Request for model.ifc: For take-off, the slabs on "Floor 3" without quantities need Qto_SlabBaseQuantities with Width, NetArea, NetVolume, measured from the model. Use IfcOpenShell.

First a look at what the model holds.

```python
import ifcopenshell
import ifcopenshell.util.element
import ifcopenshell.util.unit

model = ifcopenshell.open("model.ifc")
print(model.schema)
for unit_type in ("LENGTHUNIT", "AREAUNIT", "VOLUMEUNIT"):
    print(unit_type, ifcopenshell.util.unit.calculate_unit_scale(model, unit_type))
storey = next(s for s in model.by_type("IfcBuildingStorey") if s.Name == "Floor 3")
slabs = [e for e in ifcopenshell.util.element.get_decomposition(storey) if e.is_a("IfcSlab")]
for e in sorted(slabs, key=lambda e: e.id()):
    print(e.id(), e.is_a(), e.Name, list(ifcopenshell.util.element.get_psets(e, qtos_only=True)), sep=" | ")
```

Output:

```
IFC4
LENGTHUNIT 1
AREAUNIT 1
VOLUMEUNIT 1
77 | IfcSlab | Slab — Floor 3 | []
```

```python
import ifcopenshell
import ifcopenshell.api.pset
import ifcopenshell.geom
import ifcopenshell.util.element
import ifcopenshell.util.shape
import ifcopenshell.util.unit

model = ifcopenshell.open("model.ifc")
unit_scale = ifcopenshell.util.unit.calculate_unit_scale(model)
area_scale = ifcopenshell.util.unit.calculate_unit_scale(model, "AREAUNIT")
volume_scale = ifcopenshell.util.unit.calculate_unit_scale(model, "VOLUMEUNIT")
settings = ifcopenshell.geom.settings()

storey = next(s for s in model.by_type("IfcBuildingStorey") if s.Name == "Floor 3")
slabs = [e for e in ifcopenshell.util.element.get_decomposition(storey) if e.is_a("IfcSlab")]

for e in sorted(slabs, key=lambda e: e.id()):
    if ifcopenshell.util.element.get_psets(e, qtos_only=True, should_inherit=False):
        continue
    # Geometry comes back in metres, in the element's own axes.
    shape = ifcopenshell.geom.create_shape(settings, e)
    values = {
        "Width": ifcopenshell.util.shape.get_z(shape.geometry) / unit_scale,
        "NetArea": ifcopenshell.util.shape.get_footprint_area(shape.geometry) / area_scale,
        "NetVolume": ifcopenshell.util.shape.get_volume(shape.geometry) / volume_scale,
    }
    qto = ifcopenshell.api.pset.add_qto(model, product=e, name="Qto_SlabBaseQuantities")
    ifcopenshell.api.pset.edit_qto(model, qto=qto, properties=values)
    print(e.id(), {k: round(v, 3) for k, v in values.items()})

model.write("model_updated.ifc")
```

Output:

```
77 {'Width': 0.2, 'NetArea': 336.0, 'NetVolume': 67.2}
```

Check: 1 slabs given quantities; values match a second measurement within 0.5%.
